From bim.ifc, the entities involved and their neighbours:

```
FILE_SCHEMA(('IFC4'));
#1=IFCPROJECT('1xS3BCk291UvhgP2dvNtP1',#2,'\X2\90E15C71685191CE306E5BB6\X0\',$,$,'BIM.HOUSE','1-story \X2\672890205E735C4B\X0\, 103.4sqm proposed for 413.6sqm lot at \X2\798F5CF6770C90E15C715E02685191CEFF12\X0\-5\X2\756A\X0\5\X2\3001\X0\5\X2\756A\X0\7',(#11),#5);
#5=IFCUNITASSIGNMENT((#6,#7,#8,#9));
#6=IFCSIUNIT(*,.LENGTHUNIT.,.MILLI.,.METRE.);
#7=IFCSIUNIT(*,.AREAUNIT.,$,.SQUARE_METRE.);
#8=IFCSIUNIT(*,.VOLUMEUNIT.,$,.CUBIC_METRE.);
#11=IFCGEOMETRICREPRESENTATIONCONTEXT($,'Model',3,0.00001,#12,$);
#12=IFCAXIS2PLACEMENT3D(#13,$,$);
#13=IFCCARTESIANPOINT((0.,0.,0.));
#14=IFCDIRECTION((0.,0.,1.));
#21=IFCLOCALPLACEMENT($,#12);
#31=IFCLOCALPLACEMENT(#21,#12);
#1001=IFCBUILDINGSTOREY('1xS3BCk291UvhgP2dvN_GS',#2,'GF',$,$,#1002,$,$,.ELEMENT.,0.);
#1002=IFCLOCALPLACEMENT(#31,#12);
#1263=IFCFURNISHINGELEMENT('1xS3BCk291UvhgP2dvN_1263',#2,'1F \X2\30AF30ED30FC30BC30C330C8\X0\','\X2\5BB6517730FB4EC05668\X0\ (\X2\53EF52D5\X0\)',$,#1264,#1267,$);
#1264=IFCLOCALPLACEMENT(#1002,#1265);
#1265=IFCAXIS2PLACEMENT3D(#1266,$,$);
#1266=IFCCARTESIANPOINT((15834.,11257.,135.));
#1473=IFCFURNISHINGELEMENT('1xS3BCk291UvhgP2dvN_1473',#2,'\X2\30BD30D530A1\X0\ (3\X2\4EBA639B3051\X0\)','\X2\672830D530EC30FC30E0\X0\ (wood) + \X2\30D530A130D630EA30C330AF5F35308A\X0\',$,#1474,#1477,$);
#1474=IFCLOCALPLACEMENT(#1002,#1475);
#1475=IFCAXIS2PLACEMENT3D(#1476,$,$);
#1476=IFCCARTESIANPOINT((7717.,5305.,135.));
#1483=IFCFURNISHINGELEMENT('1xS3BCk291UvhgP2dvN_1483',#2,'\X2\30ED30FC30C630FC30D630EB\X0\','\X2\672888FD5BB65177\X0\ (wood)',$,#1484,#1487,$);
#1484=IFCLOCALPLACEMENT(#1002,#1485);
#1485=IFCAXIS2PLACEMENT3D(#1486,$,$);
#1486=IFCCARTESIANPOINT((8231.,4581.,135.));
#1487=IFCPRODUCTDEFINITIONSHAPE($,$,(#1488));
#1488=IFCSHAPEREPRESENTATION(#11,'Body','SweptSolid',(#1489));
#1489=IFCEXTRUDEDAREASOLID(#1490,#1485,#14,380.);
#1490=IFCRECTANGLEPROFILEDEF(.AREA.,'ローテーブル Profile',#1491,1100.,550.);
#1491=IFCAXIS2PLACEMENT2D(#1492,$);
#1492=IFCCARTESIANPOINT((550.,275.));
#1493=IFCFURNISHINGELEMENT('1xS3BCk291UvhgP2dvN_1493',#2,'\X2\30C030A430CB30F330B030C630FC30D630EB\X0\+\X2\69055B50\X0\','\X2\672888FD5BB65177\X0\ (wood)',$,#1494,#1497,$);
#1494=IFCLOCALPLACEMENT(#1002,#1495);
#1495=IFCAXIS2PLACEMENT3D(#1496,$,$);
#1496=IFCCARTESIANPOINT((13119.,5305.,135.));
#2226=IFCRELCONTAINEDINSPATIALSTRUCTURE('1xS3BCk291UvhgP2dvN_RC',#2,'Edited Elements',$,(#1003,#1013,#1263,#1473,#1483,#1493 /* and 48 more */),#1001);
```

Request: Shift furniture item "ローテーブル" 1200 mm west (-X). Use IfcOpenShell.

```python
import ifcopenshell
import ifcopenshell.api.geometry
import ifcopenshell.util.placement

model = ifcopenshell.open("bim.ifc")

item = model.by_id(1483)
matrix = ifcopenshell.util.placement.get_local_placement(item.ObjectPlacement)
matrix[0, 3] -= 1200.0
ifcopenshell.api.geometry.edit_object_placement(model, product=item, matrix=matrix, is_si=False)

print(ifcopenshell.util.placement.get_local_placement(item.ObjectPlacement).round(3) + 0.0)

model.write("bim_rev.ifc")
```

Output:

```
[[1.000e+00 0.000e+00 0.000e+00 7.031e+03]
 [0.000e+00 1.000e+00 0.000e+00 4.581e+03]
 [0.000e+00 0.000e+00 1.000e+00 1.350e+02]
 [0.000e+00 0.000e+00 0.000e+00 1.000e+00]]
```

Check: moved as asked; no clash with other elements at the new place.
